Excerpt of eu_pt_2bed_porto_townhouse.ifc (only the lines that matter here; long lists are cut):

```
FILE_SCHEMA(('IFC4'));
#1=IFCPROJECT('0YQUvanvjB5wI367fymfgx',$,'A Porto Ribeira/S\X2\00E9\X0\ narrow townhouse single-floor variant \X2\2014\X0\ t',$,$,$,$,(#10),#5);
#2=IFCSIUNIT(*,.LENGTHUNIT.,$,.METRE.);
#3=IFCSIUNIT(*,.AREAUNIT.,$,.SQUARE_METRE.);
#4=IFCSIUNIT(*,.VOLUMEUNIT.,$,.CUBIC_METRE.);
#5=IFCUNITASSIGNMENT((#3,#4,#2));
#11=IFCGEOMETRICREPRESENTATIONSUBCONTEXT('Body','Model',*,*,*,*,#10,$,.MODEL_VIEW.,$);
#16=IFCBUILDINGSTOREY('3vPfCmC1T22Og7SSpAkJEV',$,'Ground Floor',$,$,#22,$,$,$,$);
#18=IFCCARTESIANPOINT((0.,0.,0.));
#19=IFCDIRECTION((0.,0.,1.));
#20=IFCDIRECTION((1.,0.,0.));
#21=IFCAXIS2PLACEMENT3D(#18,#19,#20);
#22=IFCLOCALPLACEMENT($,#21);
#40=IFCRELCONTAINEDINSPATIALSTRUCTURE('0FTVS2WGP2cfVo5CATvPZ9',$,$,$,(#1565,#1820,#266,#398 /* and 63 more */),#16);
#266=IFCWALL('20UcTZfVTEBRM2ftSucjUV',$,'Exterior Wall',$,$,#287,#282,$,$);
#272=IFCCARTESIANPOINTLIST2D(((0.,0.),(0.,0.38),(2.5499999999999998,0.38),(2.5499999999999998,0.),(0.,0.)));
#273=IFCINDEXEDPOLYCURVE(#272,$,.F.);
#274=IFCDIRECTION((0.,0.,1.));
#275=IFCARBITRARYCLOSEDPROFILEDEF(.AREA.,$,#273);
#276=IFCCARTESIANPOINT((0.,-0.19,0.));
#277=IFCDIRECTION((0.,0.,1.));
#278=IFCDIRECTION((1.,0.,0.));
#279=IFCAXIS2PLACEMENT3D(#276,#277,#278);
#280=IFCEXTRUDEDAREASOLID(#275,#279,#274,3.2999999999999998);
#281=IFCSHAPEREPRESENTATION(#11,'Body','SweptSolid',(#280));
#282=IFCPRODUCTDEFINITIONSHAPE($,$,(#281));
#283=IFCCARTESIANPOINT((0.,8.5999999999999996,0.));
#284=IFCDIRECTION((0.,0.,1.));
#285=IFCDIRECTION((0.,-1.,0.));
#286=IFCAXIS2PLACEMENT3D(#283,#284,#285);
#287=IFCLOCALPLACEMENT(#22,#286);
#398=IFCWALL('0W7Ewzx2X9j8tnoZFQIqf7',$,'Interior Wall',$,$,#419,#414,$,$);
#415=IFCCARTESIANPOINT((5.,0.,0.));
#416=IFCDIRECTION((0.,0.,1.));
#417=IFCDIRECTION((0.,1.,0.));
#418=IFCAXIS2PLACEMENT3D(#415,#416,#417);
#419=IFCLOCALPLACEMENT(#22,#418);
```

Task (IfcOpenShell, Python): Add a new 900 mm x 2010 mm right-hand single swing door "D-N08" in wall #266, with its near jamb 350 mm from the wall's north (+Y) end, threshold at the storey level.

```python
import numpy as np
import ifcopenshell
import ifcopenshell.api.feature
import ifcopenshell.api.geometry
import ifcopenshell.api.root
import ifcopenshell.api.spatial
import ifcopenshell.geom
import ifcopenshell.util.element
import ifcopenshell.util.placement
import ifcopenshell.util.representation
import ifcopenshell.util.shape
import ifcopenshell.util.unit

model = ifcopenshell.open("eu_pt_2bed_porto_townhouse.ifc")
unit_scale = ifcopenshell.util.unit.calculate_unit_scale(model)
settings = ifcopenshell.geom.settings()


def volume(element):
    """Net volume in cubic metres, openings subtracted."""
    shape = ifcopenshell.geom.create_shape(settings, element)
    return ifcopenshell.util.shape.get_volume(shape.geometry)


wall = model.by_id(266)
storey = ifcopenshell.util.element.get_container(wall, ifc_class="IfcBuildingStorey")
context = ifcopenshell.util.representation.get_context(model, "Model", "Body", "MODEL_VIEW")
before = volume(wall)

width, height, from_end, sill = 0.9, 2.01, 0.35, 0.0  # metres

# The wall runs along its own X axis, and the end named is its -X end.
wall_shape = ifcopenshell.geom.create_shape(settings, wall)
x, y, z = ifcopenshell.util.shape.get_vertices(wall_shape.geometry).T
start = x.min() + from_end
face, thickness = float(y.min()), float(y.max() - y.min())
wall_matrix = ifcopenshell.util.placement.get_local_placement(wall.ObjectPlacement)
level = ifcopenshell.util.placement.get_local_placement(storey.ObjectPlacement)[2, 3]


def in_wall(x, y):
    """Placement at x, y metres in the wall's axes, at sill height."""
    matrix = wall_matrix.copy()
    matrix[:, 3] = wall_matrix @ np.array([x / unit_scale, y / unit_scale, 0.0, 1.0])
    matrix[2, 3] = level + sill / unit_scale
    return matrix


# Opening: a box that overshoots both wall faces by 50 mm.
opening = ifcopenshell.api.root.create_entity(model, ifc_class="IfcOpeningElement", predefined_type="OPENING")
box = ifcopenshell.api.geometry.add_wall_representation(
    model, context=context, length=width, height=height, thickness=thickness + 0.1
)
ifcopenshell.api.geometry.assign_representation(model, product=opening, representation=box)
ifcopenshell.api.geometry.edit_object_placement(model, product=opening, matrix=in_wall(start, face - 0.05), is_si=False)
ifcopenshell.api.feature.add_feature(model, feature=opening, element=wall)

door = ifcopenshell.api.root.create_entity(model, ifc_class="IfcDoor", name="D-N08", predefined_type="DOOR")
door.OverallWidth, door.OverallHeight = width / unit_scale, height / unit_scale
door.OperationType = "SINGLE_SWING_RIGHT"
body = ifcopenshell.api.geometry.add_door_representation(
    model,
    context=context,
    overall_width=door.OverallWidth,
    overall_height=door.OverallHeight,
    operation_type="SINGLE_SWING_RIGHT",
    lining_properties={"LiningDepth": thickness / unit_scale, "ThresholdDepth": thickness / unit_scale},
)
ifcopenshell.api.geometry.assign_representation(model, product=door, representation=body)
ifcopenshell.api.spatial.assign_container(model, products=[door], relating_structure=storey)
ifcopenshell.api.feature.add_filling(model, opening=opening, element=door)

# The lining spans the wall, so the door starts at the wall face.
ifcopenshell.api.geometry.edit_object_placement(model, product=door, matrix=in_wall(start, face), is_si=False)

after = volume(wall)

print(f"wall volume {before:.3f} -> {after:.3f} m3")

model.write("eu_pt_2bed_porto_townhouse_edited.ifc")
```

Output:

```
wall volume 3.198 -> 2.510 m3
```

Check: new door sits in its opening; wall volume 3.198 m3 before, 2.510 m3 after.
